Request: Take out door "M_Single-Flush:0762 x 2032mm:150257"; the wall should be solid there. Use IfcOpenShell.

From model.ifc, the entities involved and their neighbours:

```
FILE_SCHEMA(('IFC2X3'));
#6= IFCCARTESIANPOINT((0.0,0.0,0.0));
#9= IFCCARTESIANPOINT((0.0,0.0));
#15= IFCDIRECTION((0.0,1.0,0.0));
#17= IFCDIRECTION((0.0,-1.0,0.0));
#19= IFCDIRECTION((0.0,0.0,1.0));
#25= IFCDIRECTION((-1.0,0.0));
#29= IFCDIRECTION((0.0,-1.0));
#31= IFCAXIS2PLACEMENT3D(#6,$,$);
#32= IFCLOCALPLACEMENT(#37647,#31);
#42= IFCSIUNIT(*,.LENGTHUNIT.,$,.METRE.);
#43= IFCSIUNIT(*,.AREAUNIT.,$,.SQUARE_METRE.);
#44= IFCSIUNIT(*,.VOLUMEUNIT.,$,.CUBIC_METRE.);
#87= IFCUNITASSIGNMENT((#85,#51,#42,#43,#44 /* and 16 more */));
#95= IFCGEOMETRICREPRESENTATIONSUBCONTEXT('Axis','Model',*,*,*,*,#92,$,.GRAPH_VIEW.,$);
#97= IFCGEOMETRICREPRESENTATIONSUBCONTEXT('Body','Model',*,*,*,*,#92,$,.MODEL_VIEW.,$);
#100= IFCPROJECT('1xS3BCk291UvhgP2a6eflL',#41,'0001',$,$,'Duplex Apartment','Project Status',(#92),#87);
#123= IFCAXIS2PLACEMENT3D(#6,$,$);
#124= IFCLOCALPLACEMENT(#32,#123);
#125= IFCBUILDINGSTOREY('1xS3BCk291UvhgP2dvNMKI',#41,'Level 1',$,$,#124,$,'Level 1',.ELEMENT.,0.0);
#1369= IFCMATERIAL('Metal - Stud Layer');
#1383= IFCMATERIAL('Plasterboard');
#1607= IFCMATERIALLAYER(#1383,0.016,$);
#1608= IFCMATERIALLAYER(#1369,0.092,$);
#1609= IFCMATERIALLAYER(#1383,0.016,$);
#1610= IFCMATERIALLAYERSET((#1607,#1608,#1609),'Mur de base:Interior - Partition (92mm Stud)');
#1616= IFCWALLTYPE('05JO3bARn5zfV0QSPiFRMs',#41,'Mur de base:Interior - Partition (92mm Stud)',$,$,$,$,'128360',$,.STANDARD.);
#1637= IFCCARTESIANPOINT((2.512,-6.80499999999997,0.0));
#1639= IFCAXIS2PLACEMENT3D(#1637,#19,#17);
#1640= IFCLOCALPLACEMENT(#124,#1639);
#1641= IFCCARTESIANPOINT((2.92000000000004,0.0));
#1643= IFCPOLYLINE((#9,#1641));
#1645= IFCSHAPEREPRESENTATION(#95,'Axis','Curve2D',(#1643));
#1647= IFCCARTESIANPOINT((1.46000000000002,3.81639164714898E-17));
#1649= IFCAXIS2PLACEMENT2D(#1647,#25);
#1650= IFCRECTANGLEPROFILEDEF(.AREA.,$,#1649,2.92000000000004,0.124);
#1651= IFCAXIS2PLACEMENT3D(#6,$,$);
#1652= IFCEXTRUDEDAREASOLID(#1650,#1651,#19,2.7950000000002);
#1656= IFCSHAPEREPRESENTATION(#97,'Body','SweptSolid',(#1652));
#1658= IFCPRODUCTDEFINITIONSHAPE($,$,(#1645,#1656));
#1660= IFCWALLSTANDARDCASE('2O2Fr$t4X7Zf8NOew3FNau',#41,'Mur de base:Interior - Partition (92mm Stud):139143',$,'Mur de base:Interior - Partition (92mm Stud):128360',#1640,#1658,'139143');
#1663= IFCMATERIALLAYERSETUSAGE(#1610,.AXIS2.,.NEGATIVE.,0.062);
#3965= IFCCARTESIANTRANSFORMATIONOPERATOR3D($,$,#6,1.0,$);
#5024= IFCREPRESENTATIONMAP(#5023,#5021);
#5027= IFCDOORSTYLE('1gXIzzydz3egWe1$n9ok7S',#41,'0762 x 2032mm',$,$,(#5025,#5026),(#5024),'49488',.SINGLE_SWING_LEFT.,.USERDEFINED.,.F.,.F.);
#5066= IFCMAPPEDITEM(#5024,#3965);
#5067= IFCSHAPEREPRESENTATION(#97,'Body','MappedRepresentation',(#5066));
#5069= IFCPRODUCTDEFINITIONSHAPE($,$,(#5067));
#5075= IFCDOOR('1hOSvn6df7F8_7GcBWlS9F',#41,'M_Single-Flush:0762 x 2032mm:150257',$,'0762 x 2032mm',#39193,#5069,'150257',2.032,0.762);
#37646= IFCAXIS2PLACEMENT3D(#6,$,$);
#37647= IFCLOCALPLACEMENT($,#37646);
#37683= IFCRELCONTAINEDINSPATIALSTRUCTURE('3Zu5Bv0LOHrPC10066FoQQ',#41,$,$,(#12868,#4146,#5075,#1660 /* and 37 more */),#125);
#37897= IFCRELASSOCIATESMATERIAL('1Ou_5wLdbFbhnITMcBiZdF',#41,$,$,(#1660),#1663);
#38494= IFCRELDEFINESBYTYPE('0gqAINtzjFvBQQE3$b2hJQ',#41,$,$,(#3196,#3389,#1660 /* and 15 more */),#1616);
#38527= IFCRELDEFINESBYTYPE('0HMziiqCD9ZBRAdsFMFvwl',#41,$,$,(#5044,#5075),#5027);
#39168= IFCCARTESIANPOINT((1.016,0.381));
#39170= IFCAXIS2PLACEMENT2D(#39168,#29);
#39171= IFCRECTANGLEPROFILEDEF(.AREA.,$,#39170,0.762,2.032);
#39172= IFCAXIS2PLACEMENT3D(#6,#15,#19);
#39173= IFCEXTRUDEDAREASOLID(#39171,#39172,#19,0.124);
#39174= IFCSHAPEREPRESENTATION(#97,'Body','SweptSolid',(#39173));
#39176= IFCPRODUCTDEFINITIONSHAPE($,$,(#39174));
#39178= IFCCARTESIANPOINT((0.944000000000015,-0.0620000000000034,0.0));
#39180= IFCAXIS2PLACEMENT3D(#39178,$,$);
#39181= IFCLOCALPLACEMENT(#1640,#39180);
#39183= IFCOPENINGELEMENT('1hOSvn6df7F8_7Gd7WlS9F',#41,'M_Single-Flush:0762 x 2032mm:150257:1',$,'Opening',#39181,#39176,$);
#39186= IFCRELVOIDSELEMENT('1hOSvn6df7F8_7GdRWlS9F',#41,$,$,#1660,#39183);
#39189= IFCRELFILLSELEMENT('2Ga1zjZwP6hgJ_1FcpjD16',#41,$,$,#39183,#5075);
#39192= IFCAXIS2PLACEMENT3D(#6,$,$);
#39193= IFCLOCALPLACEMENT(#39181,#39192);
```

```python
import ifcopenshell
import ifcopenshell.api.feature
import ifcopenshell.api.root
import ifcopenshell.geom
import ifcopenshell.util.shape

model = ifcopenshell.open("model.ifc")
settings = ifcopenshell.geom.settings()


def volume(element):
    """Net volume in cubic metres, openings subtracted."""
    shape = ifcopenshell.geom.create_shape(settings, element)
    return ifcopenshell.util.shape.get_volume(shape.geometry)


door = model.by_id(5075)
opening = door.FillsVoids[0].RelatingOpeningElement
wall = opening.VoidsElements[0].RelatingBuildingElement
before = volume(wall)

ifcopenshell.api.root.remove_product(model, product=door)
ifcopenshell.api.feature.remove_feature(model, feature=opening)

after = volume(wall)

print(f"wall volume {before:.3f} -> {after:.3f} m3")

model.write("model-out.ifc")
```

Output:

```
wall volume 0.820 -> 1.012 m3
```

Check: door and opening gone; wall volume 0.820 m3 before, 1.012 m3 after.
